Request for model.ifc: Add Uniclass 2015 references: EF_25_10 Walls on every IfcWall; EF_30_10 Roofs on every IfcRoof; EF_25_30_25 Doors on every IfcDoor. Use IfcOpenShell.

First a look at what the model holds.

```python
import ifcopenshell

model = ifcopenshell.open("model.ifc")
print(model.schema)
print("classifications:", [c.Name for c in model.by_type("IfcClassification")])
for ifc_class in ("IfcDoor", "IfcRoof", "IfcStair", "IfcWall", "IfcWindow"):
    print(ifc_class, len(model.by_type(ifc_class)))
```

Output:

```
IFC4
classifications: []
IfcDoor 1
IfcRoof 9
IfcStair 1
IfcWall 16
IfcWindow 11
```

```python
import ifcopenshell
import ifcopenshell.api.classification

model = ifcopenshell.open("model.ifc")

system = ifcopenshell.api.classification.add_classification(model, classification="Uniclass 2015")

codes = {
    "IfcWall": ("EF_25_10", "Walls"),
    "IfcRoof": ("EF_30_10", "Roofs"),
    "IfcDoor": ("EF_25_30_25", "Doors"),
}
for ifc_class, (code, name) in codes.items():
    products = model.by_type(ifc_class)
    ifcopenshell.api.classification.add_reference(
        model, products=products, classification=system, identification=code, name=name
    )
    print(code, len(products))

model.write("model_edited.ifc")
```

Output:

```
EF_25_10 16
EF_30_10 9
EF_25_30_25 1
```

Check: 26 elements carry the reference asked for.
